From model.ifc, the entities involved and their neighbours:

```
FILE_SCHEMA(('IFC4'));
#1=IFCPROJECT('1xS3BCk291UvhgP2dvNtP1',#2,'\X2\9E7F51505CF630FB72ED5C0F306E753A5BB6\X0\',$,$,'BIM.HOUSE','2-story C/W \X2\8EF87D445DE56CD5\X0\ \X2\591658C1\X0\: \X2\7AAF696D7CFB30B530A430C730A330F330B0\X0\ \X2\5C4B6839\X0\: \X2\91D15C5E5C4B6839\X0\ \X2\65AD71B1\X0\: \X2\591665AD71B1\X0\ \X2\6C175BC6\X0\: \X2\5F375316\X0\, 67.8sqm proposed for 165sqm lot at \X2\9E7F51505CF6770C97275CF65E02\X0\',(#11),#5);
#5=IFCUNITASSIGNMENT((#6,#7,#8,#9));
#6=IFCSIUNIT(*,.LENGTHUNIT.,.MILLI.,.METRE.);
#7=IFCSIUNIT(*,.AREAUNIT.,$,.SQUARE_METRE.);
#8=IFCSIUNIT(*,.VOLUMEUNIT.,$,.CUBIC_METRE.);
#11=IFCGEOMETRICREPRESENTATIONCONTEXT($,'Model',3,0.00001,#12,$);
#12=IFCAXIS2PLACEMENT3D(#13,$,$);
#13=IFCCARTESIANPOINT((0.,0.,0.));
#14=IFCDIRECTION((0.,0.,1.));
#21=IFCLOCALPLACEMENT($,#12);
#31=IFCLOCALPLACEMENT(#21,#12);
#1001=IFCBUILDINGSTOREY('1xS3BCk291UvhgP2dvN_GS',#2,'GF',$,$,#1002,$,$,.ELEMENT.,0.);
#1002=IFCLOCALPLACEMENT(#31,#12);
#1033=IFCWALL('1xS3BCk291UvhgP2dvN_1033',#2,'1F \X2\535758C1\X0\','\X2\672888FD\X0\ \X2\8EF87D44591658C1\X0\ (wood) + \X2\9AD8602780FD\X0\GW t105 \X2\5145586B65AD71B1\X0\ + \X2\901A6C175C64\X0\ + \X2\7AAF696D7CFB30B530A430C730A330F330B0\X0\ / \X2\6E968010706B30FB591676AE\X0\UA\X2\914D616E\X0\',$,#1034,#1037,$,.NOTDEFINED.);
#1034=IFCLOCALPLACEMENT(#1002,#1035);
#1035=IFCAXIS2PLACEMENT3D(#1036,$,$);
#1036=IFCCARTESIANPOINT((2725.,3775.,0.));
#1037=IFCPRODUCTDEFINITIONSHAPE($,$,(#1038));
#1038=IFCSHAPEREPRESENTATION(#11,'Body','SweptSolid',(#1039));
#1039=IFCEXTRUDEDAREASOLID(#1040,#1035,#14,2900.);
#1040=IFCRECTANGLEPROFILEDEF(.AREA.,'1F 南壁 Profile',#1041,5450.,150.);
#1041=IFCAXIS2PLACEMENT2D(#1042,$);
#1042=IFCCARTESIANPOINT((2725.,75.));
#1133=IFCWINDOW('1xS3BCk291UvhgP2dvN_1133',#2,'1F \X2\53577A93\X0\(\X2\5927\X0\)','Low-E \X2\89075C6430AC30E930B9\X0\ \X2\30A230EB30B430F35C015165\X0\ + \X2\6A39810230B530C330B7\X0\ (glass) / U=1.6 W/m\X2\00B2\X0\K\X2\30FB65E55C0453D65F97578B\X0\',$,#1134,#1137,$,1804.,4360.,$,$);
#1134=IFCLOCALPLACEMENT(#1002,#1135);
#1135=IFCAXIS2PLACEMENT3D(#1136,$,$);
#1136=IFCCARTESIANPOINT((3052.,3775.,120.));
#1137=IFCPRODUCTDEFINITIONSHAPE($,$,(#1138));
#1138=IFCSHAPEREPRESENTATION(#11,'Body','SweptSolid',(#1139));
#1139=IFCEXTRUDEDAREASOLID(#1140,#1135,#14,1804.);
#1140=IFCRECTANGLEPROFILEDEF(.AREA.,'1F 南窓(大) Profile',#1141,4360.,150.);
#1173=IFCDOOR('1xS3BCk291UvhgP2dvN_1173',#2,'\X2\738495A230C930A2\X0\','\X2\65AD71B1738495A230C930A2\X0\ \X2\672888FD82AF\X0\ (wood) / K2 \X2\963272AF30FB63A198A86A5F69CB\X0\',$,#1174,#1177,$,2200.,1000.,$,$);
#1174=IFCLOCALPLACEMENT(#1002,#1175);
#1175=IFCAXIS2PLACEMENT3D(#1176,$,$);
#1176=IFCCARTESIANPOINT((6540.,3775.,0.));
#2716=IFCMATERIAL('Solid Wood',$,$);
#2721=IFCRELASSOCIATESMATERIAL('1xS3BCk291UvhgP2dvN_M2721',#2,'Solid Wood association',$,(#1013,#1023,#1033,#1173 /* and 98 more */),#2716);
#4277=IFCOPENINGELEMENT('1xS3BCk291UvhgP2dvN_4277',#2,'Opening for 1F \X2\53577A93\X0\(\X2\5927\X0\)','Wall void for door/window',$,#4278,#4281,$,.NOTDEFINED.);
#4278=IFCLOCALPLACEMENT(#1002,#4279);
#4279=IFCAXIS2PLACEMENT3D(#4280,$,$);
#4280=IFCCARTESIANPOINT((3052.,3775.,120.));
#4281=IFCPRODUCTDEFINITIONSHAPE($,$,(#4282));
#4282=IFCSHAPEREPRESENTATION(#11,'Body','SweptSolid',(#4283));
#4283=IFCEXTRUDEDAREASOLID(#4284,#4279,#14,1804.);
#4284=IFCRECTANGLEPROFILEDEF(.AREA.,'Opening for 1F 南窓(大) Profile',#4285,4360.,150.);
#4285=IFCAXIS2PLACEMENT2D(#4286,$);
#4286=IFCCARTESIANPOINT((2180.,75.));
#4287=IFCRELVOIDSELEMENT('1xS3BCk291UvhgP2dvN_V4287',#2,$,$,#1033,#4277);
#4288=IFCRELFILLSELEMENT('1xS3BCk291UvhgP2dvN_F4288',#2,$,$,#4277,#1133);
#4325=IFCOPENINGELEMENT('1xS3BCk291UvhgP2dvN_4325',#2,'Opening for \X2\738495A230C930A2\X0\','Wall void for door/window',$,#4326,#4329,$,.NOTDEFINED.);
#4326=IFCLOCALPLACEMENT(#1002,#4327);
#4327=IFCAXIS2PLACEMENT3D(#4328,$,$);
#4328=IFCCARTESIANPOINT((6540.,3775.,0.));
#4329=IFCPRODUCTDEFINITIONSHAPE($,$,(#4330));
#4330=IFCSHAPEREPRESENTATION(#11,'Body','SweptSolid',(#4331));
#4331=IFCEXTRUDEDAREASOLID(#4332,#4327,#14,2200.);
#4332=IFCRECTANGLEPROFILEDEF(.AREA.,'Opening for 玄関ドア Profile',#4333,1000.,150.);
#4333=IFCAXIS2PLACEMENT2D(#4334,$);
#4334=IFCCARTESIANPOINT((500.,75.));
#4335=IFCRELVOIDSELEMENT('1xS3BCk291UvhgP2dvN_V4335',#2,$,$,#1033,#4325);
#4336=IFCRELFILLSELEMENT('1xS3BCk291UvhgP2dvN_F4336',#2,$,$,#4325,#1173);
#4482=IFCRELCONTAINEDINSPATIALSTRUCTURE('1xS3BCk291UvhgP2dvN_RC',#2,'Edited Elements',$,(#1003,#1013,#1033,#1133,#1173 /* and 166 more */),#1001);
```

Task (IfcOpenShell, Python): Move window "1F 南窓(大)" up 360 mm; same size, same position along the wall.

```python
import numpy as np
import ifcopenshell
import ifcopenshell.api.geometry
import ifcopenshell.util.placement
import ifcopenshell.util.unit

model = ifcopenshell.open("model.ifc")
unit_scale = ifcopenshell.util.unit.calculate_unit_scale(model)

window = model.by_id(1133)
opening = window.FillsVoids[0].RelatingOpeningElement
dz = 360.0

shift = np.array([0.0, 0.0, dz])
# The window is not placed relative to its opening, so move both.
for product in (opening, window):
    matrix = ifcopenshell.util.placement.get_local_placement(product.ObjectPlacement)
    matrix[:3, 3] += shift
    ifcopenshell.api.geometry.edit_object_placement(model, product=product, matrix=matrix, is_si=False)

print(f"moved by {dz * unit_scale:+.3f} m")

model.write("model_rev.ifc")
```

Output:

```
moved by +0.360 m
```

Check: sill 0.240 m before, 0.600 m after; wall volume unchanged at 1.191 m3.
